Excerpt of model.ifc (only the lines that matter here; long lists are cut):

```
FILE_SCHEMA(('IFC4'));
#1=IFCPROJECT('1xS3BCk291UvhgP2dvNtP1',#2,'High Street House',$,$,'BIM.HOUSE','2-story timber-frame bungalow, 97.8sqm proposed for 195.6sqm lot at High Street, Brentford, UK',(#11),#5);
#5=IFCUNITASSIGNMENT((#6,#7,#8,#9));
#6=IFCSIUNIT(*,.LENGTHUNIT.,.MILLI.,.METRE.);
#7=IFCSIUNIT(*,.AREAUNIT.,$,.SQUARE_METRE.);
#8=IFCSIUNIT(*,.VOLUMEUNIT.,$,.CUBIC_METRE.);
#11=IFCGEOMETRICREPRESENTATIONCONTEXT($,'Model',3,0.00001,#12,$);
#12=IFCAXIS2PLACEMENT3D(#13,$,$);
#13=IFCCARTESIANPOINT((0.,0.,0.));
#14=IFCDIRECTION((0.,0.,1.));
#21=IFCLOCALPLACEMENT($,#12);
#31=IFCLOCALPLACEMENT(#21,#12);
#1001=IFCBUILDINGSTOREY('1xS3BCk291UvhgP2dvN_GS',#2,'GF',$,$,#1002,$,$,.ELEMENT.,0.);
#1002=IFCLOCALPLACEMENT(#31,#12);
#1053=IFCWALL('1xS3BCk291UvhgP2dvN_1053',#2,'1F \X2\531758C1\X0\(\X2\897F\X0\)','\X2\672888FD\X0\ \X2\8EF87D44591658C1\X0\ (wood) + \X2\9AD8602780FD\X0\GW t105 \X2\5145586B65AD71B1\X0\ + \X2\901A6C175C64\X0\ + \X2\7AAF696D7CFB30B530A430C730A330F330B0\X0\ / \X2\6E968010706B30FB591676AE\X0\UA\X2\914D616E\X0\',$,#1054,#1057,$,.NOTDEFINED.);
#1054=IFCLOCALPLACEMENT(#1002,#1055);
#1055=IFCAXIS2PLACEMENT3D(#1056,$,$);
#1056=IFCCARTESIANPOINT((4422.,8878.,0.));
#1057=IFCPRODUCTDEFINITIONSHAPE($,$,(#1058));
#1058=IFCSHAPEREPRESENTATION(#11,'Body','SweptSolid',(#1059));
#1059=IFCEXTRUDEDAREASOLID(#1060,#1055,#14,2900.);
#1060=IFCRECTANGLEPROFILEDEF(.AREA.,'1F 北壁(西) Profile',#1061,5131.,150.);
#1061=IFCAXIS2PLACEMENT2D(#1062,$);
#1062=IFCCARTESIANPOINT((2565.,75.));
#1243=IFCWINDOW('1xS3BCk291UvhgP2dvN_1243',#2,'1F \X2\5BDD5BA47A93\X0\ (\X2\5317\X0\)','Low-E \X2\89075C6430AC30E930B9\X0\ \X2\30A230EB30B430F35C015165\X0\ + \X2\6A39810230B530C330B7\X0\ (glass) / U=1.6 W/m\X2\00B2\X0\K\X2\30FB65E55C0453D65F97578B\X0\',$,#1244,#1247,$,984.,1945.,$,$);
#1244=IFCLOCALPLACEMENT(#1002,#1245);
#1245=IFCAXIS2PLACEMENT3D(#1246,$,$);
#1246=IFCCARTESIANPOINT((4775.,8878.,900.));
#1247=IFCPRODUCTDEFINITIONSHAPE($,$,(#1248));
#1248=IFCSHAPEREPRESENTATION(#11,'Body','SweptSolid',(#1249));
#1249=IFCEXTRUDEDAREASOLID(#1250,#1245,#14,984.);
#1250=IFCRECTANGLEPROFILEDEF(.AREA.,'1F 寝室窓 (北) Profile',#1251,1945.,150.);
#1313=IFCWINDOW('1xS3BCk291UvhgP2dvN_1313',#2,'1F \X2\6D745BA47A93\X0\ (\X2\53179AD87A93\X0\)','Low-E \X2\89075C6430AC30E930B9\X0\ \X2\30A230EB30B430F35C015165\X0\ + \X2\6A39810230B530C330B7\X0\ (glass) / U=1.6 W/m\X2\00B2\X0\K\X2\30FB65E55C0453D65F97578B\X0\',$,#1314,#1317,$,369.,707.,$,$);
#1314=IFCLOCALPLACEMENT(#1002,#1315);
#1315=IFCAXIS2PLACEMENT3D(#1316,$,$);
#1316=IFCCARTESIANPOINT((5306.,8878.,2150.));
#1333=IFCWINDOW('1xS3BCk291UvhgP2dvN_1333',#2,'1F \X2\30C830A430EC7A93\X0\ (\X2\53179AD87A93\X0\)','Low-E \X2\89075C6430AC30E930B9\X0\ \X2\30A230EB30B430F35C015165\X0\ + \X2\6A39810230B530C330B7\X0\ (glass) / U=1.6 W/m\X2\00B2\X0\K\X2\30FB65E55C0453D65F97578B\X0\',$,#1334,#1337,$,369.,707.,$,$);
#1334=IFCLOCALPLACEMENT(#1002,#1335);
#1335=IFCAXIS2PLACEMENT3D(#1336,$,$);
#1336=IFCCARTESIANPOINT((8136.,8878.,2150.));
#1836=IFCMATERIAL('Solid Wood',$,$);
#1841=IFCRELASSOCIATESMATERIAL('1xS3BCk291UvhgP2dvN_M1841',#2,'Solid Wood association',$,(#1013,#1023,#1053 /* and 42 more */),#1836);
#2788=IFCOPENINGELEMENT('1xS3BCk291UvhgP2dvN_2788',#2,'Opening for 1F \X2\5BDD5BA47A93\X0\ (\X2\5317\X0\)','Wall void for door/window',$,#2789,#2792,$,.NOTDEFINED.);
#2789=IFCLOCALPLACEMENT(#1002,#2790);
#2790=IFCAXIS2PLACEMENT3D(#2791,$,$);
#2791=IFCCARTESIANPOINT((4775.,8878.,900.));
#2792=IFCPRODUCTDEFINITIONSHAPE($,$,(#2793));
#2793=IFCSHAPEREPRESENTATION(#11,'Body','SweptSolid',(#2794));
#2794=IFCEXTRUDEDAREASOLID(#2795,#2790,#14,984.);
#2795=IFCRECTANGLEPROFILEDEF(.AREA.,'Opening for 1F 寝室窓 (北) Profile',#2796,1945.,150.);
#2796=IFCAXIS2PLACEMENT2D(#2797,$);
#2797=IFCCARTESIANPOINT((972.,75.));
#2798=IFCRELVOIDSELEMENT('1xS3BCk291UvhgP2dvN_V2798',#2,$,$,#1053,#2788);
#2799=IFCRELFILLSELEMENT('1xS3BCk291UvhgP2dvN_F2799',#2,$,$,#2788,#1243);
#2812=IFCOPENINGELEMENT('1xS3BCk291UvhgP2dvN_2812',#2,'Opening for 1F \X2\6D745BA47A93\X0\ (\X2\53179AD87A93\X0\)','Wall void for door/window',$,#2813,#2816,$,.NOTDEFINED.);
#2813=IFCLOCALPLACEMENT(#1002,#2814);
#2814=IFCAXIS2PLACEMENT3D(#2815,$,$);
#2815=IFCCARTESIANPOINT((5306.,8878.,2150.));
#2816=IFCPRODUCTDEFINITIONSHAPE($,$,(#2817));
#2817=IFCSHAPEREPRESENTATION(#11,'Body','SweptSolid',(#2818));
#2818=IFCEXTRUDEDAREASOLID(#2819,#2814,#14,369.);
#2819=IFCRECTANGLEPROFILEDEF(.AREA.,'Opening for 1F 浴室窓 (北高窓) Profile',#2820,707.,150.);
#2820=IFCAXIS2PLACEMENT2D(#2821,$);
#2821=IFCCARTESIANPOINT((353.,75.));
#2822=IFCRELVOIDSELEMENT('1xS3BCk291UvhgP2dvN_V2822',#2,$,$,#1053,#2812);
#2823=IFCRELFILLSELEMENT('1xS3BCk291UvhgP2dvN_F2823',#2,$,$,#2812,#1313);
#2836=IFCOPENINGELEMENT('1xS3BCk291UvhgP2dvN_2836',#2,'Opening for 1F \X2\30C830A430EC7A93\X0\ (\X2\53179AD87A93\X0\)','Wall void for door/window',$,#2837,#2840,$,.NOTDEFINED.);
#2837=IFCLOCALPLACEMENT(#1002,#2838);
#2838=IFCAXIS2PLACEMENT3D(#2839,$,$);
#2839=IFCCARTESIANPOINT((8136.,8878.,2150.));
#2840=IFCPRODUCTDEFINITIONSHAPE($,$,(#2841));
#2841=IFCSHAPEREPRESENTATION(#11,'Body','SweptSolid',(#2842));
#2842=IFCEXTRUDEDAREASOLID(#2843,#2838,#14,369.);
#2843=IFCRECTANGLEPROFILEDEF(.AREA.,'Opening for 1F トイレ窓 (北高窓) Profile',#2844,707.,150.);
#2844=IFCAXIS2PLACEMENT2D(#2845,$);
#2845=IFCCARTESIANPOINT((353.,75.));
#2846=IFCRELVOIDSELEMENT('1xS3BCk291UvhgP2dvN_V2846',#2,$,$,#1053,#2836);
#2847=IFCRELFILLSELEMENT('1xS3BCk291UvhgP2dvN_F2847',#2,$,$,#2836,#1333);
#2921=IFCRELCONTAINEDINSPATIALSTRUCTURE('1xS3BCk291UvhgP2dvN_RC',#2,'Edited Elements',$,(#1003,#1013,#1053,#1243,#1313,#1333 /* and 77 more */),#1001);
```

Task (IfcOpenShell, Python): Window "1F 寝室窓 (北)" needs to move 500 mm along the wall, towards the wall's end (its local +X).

```python
import ifcopenshell
import ifcopenshell.api.geometry
import ifcopenshell.util.placement

model = ifcopenshell.open("model.ifc")

window = model.by_guid("1xS3BCk291UvhgP2dvN_1243")
opening = window.FillsVoids[0].RelatingOpeningElement
wall = opening.VoidsElements[0].RelatingBuildingElement

wall_matrix = ifcopenshell.util.placement.get_local_placement(wall.ObjectPlacement)
shift = wall_matrix[:3, 0] * 500.0
before = ifcopenshell.util.placement.get_local_placement(window.ObjectPlacement)[:3, 3].copy()

# The window is not placed relative to its opening, so move both.
for product in (opening, window):
    matrix = ifcopenshell.util.placement.get_local_placement(product.ObjectPlacement)
    matrix[:3, 3] += shift
    ifcopenshell.api.geometry.edit_object_placement(model, product=product, matrix=matrix, is_si=False)

after = ifcopenshell.util.placement.get_local_placement(window.ObjectPlacement)[:3, 3]
print("window moved by", (after - before).round(3) + 0.0)

model.write("model_v2.ifc")
```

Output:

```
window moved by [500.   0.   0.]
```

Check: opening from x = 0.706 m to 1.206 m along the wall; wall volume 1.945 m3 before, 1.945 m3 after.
